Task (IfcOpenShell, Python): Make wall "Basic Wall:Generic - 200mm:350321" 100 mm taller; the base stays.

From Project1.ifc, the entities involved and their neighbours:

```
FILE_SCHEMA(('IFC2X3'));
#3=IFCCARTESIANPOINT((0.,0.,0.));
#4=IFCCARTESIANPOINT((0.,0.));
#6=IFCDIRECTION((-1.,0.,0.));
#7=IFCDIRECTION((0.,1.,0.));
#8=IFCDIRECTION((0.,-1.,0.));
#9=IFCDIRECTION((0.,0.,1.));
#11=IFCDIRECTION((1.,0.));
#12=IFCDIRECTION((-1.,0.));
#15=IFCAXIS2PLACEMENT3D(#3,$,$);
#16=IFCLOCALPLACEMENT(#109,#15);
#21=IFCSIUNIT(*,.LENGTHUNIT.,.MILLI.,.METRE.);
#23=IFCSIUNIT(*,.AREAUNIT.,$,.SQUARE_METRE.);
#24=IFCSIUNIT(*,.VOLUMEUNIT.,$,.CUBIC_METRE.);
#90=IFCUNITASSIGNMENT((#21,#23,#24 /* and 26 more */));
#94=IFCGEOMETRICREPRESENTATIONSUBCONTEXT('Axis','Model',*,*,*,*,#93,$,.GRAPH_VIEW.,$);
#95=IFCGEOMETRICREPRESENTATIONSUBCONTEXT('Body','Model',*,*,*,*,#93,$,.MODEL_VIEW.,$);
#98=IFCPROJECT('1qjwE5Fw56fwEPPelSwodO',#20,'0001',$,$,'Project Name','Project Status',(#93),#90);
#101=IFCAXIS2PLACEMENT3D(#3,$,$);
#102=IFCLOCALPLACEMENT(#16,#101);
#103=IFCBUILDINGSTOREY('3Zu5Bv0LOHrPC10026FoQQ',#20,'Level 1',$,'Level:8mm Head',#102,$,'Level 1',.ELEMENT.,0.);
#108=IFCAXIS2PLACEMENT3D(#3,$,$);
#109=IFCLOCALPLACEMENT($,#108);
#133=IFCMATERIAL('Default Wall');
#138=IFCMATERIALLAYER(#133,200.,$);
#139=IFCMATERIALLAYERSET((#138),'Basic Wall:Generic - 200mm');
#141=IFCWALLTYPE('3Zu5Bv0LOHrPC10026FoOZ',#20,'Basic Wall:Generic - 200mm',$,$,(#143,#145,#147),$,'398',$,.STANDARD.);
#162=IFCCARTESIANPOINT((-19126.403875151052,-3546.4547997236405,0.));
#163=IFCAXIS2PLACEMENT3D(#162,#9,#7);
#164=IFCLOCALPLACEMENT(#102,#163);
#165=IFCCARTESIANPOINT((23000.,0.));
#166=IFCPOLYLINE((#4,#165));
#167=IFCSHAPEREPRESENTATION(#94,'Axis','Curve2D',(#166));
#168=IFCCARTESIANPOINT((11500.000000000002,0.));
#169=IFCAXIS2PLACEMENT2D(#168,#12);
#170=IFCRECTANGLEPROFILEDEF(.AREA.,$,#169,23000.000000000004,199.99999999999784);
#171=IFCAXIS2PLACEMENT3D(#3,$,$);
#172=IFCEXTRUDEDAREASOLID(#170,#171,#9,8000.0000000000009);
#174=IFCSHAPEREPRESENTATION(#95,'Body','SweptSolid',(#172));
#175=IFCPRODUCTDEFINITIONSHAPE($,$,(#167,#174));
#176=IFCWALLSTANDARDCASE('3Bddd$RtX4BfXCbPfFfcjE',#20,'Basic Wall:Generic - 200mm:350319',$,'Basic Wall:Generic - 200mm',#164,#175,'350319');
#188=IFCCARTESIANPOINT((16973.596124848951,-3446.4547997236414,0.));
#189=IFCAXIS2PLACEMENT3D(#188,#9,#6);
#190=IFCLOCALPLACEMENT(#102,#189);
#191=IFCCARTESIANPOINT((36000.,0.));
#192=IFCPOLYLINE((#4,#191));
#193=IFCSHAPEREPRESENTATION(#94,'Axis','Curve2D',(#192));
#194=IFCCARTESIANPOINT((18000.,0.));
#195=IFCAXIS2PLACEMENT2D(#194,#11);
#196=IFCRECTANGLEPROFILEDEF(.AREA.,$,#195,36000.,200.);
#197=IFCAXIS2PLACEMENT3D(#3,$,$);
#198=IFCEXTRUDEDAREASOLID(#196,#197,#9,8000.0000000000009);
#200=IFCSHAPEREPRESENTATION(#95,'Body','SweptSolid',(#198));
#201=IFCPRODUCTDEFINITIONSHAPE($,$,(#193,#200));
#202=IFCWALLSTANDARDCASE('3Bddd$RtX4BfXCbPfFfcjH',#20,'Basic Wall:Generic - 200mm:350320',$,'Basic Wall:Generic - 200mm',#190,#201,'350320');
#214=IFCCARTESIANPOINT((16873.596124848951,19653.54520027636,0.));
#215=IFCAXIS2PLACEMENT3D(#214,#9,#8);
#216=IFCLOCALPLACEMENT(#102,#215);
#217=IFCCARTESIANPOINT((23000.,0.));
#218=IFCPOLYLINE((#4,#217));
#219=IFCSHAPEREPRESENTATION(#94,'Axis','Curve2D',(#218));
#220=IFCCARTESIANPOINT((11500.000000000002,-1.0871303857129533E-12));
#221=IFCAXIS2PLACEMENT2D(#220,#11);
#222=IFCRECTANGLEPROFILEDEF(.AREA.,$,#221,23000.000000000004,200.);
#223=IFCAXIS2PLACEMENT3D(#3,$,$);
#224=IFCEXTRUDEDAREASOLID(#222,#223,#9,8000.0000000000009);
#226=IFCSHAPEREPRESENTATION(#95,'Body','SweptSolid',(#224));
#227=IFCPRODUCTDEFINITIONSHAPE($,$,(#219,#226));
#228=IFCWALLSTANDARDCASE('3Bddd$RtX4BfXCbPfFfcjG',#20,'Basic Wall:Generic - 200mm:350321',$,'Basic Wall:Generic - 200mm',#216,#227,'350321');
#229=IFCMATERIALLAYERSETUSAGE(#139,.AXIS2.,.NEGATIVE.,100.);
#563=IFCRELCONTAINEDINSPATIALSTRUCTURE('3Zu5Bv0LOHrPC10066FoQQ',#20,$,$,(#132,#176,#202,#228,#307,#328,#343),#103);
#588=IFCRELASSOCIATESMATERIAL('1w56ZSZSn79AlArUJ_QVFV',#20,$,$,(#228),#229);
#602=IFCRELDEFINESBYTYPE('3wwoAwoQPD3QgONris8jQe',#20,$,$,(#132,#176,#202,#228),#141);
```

```python
import ifcopenshell
import ifcopenshell.geom
import ifcopenshell.util.representation
import ifcopenshell.util.shape

model = ifcopenshell.open("Project1.ifc")
settings = ifcopenshell.geom.settings()


def volume(element):
    """Net volume in cubic metres, openings subtracted."""
    shape = ifcopenshell.geom.create_shape(settings, element)
    return ifcopenshell.util.shape.get_volume(shape.geometry)


wall = model.by_guid("3Bddd$RtX4BfXCbPfFfcjG")
before = volume(wall)

body = ifcopenshell.util.representation.get_representation(wall, "Model", "Body")
solid = body.Items[0]
old_height = solid.Depth
solid.Depth += 100.0
after = volume(wall)

print(f"height {old_height:g} -> {solid.Depth:g}, volume {before:.3f} -> {after:.3f} m3")

model.write("Project1_rev.ifc")
```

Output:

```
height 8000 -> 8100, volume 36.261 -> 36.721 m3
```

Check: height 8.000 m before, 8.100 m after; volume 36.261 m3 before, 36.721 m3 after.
